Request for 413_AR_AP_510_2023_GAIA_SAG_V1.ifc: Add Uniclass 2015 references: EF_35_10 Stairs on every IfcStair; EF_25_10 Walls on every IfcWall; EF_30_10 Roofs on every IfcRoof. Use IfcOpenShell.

First a look at what the model holds.

```python
import ifcopenshell

model = ifcopenshell.open("413_AR_AP_510_2023_GAIA_SAG_V1.ifc")
print(model.schema)
print("classifications:", [c.Name for c in model.by_type("IfcClassification")])
for ifc_class in ("IfcDoor", "IfcRoof", "IfcStair", "IfcWall", "IfcWindow"):
    print(ifc_class, len(model.by_type(ifc_class)))
```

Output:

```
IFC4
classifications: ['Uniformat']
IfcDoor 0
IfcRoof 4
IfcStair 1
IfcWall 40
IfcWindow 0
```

```python
import ifcopenshell
import ifcopenshell.api.classification

model = ifcopenshell.open("413_AR_AP_510_2023_GAIA_SAG_V1.ifc")

system = ifcopenshell.api.classification.add_classification(model, classification="Uniclass 2015")

codes = {
    "IfcStair": ("EF_35_10", "Stairs"),
    "IfcWall": ("EF_25_10", "Walls"),
    "IfcRoof": ("EF_30_10", "Roofs"),
}
for ifc_class, (code, name) in codes.items():
    products = model.by_type(ifc_class)
    ifcopenshell.api.classification.add_reference(
        model, products=products, classification=system, identification=code, name=name
    )
    print(code, len(products))

model.write("413_AR_AP_510_2023_GAIA_SAG_V1_edited.ifc")
```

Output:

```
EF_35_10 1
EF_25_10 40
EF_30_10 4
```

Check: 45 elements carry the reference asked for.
